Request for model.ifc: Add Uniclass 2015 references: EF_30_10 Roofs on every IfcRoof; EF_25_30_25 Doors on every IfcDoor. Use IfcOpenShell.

First a look at what the model holds.

```python
import ifcopenshell

model = ifcopenshell.open("model.ifc")
print(model.schema)
print("classifications:", [c.Name for c in model.by_type("IfcClassification")])
for ifc_class in ("IfcDoor", "IfcRoof", "IfcStair", "IfcWall", "IfcWindow"):
    print(ifc_class, len(model.by_type(ifc_class)))
```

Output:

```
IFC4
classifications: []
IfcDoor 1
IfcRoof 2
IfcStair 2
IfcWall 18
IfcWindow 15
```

```python
import ifcopenshell
import ifcopenshell.api.classification

model = ifcopenshell.open("model.ifc")

system = ifcopenshell.api.classification.add_classification(model, classification="Uniclass 2015")

codes = {
    "IfcRoof": ("EF_30_10", "Roofs"),
    "IfcDoor": ("EF_25_30_25", "Doors"),
}
for ifc_class, (code, name) in codes.items():
    products = model.by_type(ifc_class)
    ifcopenshell.api.classification.add_reference(
        model, products=products, classification=system, identification=code, name=name
    )
    print(code, len(products))

model.write("model_updated.ifc")
```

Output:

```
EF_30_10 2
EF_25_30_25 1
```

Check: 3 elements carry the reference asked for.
